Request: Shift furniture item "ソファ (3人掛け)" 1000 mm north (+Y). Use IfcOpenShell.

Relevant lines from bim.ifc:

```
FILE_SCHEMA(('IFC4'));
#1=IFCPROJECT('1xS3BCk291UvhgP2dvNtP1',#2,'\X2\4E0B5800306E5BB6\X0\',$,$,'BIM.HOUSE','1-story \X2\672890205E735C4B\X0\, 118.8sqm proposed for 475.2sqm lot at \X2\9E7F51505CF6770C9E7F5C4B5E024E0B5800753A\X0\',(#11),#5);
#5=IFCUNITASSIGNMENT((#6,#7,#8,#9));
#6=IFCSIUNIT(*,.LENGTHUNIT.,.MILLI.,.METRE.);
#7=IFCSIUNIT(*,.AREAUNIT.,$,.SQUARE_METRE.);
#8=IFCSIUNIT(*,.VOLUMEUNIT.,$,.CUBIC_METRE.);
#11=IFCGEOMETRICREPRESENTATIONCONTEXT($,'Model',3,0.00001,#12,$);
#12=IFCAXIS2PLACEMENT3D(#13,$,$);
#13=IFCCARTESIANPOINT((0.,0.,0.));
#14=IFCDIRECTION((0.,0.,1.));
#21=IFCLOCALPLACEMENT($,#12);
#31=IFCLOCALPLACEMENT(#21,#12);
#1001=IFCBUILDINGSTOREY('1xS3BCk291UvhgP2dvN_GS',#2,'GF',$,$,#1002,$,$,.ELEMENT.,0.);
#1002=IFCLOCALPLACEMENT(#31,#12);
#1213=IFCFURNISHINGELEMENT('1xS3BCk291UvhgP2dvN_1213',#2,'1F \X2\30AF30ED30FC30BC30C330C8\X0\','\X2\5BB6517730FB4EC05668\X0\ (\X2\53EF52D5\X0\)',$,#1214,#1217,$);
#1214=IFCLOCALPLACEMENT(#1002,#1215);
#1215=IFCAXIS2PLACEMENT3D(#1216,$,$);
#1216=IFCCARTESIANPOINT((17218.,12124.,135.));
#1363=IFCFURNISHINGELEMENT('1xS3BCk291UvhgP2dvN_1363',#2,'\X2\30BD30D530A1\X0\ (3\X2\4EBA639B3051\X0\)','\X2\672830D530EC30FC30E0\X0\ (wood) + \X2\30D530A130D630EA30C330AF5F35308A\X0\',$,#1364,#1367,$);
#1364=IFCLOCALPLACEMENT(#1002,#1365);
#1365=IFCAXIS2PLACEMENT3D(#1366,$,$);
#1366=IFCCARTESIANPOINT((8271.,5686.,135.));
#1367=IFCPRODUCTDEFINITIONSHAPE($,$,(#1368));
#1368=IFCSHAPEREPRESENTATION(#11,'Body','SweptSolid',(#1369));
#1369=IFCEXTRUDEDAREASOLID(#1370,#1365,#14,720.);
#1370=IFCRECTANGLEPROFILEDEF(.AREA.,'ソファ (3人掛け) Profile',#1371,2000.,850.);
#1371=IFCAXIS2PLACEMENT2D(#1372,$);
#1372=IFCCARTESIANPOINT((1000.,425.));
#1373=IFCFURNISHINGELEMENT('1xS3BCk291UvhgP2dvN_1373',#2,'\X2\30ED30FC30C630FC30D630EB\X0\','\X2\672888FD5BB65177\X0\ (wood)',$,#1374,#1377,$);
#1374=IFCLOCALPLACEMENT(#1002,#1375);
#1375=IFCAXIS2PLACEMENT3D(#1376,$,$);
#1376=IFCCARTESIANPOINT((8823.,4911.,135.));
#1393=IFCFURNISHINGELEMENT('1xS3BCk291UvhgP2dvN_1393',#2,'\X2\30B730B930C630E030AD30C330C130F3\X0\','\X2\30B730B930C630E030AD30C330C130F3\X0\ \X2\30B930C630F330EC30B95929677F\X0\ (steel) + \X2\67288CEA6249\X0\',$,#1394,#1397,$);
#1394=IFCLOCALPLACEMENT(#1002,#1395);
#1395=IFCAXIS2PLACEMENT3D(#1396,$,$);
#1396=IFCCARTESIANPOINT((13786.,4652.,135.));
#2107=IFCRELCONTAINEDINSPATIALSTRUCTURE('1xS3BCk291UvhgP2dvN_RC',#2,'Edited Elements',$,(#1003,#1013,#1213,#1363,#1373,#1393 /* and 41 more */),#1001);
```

```python
import ifcopenshell
import ifcopenshell.api.geometry
import ifcopenshell.util.placement
import ifcopenshell.util.unit

model = ifcopenshell.open("bim.ifc")
unit_scale = ifcopenshell.util.unit.calculate_unit_scale(model)

item = model.by_guid("1xS3BCk291UvhgP2dvN_1363")
matrix = ifcopenshell.util.placement.get_local_placement(item.ObjectPlacement)
matrix[1, 3] += 1 / unit_scale
ifcopenshell.api.geometry.edit_object_placement(model, product=item, matrix=matrix, is_si=False)

print(ifcopenshell.util.placement.get_local_placement(item.ObjectPlacement).round(3) + 0.0)

model.write("bim_updated.ifc")
```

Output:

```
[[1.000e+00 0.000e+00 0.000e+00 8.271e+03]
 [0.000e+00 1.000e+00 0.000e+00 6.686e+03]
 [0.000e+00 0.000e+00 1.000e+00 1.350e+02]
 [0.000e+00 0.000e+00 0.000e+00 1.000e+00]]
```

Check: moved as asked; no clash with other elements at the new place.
